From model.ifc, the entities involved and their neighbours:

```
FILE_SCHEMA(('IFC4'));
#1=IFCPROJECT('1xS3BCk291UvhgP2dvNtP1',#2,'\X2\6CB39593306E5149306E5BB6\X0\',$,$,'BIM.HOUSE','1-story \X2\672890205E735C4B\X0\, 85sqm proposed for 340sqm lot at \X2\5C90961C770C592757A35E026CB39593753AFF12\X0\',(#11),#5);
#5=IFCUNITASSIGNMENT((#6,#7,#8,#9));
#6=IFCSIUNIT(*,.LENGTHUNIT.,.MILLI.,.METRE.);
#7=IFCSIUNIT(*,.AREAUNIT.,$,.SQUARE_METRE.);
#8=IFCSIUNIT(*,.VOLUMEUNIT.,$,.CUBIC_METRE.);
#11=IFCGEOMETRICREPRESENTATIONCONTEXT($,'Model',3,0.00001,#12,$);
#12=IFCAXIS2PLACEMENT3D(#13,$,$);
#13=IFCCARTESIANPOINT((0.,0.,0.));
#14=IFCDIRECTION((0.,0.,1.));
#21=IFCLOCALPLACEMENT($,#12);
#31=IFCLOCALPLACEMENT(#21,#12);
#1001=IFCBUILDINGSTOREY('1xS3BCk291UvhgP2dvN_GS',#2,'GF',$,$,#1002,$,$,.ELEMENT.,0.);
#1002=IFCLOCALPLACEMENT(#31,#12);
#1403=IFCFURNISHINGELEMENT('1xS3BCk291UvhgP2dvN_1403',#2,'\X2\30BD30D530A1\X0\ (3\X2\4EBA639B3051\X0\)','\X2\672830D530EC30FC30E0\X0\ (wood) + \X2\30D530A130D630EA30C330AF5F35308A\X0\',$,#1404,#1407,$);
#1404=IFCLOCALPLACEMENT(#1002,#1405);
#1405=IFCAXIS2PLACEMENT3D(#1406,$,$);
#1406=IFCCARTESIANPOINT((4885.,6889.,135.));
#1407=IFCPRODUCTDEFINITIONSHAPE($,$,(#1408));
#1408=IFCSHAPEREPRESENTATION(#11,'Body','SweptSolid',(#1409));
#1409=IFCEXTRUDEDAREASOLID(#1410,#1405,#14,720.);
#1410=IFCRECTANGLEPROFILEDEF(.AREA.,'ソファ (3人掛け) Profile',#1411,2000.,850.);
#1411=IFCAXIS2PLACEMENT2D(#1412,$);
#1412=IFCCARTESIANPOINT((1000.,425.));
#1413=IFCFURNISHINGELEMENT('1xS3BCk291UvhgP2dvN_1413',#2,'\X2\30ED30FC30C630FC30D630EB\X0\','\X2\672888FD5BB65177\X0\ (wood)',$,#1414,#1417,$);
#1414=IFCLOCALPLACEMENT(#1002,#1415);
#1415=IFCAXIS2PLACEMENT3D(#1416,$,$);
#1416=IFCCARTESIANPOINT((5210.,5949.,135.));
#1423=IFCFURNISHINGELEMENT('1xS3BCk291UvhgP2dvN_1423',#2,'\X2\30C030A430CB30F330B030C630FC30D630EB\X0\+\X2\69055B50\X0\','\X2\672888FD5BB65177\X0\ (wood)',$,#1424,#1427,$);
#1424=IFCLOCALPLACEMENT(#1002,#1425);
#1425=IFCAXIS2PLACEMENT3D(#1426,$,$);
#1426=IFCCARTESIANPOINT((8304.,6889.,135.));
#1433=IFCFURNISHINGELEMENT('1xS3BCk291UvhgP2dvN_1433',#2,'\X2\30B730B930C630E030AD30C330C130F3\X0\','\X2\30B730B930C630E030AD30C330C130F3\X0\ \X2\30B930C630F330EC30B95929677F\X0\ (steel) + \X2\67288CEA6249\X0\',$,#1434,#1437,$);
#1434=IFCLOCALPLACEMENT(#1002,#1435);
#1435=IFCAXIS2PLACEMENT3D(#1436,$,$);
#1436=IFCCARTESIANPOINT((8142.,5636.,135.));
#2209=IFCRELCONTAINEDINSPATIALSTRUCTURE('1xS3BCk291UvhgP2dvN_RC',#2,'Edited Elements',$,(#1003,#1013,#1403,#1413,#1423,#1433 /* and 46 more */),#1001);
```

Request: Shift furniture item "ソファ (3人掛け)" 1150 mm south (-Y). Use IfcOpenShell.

```python
import ifcopenshell
import ifcopenshell.api.geometry
import ifcopenshell.util.placement
import ifcopenshell.util.unit

model = ifcopenshell.open("model.ifc")
unit_scale = ifcopenshell.util.unit.calculate_unit_scale(model)

item = model.by_guid("1xS3BCk291UvhgP2dvN_1403")
matrix = ifcopenshell.util.placement.get_local_placement(item.ObjectPlacement)
matrix[1, 3] -= 1.15 / unit_scale
ifcopenshell.api.geometry.edit_object_placement(model, product=item, matrix=matrix, is_si=False)

print(ifcopenshell.util.placement.get_local_placement(item.ObjectPlacement).round(3) + 0.0)

model.write("model_rev.ifc")
```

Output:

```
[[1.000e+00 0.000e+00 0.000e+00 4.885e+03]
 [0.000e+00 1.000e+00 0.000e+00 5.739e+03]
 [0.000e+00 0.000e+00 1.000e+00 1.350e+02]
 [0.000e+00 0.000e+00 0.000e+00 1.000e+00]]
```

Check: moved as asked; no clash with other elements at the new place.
